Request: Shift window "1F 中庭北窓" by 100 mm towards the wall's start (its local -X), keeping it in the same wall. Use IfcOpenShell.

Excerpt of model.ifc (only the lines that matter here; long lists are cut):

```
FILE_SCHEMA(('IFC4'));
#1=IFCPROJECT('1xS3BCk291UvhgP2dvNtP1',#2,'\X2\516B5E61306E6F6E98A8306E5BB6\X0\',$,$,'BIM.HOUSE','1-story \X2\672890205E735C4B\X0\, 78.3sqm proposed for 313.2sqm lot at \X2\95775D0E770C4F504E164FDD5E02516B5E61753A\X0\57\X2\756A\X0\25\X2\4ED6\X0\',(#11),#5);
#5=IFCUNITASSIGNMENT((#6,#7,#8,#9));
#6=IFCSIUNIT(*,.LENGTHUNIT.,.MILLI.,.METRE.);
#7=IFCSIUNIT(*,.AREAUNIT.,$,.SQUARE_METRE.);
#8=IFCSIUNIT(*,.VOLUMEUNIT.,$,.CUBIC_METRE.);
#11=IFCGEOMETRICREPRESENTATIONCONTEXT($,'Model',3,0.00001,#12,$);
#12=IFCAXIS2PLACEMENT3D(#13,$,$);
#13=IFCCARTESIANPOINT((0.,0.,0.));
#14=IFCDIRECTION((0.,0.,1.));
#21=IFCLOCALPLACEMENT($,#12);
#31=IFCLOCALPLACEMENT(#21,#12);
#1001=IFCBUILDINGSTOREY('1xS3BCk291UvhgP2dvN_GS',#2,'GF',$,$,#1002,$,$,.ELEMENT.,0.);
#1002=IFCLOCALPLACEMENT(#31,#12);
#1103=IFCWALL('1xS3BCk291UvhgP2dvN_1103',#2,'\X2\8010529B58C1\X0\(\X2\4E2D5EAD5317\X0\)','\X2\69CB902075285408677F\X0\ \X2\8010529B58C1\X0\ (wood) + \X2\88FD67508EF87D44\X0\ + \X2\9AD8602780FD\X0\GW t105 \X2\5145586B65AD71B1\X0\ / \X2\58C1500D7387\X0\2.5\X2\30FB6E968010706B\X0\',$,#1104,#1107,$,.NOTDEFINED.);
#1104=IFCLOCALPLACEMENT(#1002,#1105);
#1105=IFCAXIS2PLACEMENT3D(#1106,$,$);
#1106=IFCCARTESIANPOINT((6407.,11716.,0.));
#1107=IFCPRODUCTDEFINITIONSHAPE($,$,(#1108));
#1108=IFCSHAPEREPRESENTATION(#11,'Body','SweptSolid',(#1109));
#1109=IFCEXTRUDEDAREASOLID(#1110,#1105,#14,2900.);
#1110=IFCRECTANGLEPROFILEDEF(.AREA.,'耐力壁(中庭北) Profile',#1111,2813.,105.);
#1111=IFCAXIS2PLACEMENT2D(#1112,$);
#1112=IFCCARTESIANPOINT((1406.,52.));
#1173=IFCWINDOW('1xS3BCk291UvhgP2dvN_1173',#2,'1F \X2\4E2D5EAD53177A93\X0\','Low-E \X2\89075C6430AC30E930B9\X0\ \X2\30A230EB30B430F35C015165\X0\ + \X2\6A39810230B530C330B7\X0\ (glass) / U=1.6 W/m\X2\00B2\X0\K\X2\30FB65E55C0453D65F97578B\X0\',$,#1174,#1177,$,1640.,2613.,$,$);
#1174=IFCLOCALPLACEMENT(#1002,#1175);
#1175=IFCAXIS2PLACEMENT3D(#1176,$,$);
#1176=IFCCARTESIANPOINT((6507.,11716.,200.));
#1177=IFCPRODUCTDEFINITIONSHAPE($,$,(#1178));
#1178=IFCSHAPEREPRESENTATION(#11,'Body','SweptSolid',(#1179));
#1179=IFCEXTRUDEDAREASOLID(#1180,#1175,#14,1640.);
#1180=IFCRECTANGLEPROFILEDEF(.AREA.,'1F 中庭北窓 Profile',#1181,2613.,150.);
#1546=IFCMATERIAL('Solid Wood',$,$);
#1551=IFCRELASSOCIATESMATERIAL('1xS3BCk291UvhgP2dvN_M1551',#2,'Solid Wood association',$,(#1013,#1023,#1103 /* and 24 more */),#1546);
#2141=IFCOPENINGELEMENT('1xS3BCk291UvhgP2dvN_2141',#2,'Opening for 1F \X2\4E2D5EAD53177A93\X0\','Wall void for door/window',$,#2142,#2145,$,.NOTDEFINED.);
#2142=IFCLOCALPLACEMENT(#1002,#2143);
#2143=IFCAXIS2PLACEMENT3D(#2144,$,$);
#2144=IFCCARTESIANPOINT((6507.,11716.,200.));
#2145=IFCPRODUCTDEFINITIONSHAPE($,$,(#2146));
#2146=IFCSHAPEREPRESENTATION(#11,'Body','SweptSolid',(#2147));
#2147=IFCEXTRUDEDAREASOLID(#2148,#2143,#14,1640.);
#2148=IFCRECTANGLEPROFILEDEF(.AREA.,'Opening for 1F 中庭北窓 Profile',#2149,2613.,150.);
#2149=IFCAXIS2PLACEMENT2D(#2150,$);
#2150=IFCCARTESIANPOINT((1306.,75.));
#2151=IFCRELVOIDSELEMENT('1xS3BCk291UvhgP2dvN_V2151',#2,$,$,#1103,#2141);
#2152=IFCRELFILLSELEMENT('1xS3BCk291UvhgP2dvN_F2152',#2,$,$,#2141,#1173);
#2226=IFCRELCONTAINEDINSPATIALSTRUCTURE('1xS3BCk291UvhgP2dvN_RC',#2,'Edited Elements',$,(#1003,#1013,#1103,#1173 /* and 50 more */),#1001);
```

```python
import ifcopenshell
import ifcopenshell.api.geometry
import ifcopenshell.util.placement

model = ifcopenshell.open("model.ifc")

window = model.by_id(1173)
opening = window.FillsVoids[0].RelatingOpeningElement
wall = opening.VoidsElements[0].RelatingBuildingElement

wall_matrix = ifcopenshell.util.placement.get_local_placement(wall.ObjectPlacement)
shift = wall_matrix[:3, 0] * -100.0
before = ifcopenshell.util.placement.get_local_placement(window.ObjectPlacement)[:3, 3].copy()

# The window is not placed relative to its opening, so move both.
for product in (opening, window):
    matrix = ifcopenshell.util.placement.get_local_placement(product.ObjectPlacement)
    matrix[:3, 3] += shift
    ifcopenshell.api.geometry.edit_object_placement(model, product=product, matrix=matrix, is_si=False)

after = ifcopenshell.util.placement.get_local_placement(window.ObjectPlacement)[:3, 3]
print("window moved by", (after - before).round(3) + 0.0)

model.write("model-out.ifc")
```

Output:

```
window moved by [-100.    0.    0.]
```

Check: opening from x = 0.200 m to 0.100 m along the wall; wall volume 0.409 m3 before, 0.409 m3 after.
